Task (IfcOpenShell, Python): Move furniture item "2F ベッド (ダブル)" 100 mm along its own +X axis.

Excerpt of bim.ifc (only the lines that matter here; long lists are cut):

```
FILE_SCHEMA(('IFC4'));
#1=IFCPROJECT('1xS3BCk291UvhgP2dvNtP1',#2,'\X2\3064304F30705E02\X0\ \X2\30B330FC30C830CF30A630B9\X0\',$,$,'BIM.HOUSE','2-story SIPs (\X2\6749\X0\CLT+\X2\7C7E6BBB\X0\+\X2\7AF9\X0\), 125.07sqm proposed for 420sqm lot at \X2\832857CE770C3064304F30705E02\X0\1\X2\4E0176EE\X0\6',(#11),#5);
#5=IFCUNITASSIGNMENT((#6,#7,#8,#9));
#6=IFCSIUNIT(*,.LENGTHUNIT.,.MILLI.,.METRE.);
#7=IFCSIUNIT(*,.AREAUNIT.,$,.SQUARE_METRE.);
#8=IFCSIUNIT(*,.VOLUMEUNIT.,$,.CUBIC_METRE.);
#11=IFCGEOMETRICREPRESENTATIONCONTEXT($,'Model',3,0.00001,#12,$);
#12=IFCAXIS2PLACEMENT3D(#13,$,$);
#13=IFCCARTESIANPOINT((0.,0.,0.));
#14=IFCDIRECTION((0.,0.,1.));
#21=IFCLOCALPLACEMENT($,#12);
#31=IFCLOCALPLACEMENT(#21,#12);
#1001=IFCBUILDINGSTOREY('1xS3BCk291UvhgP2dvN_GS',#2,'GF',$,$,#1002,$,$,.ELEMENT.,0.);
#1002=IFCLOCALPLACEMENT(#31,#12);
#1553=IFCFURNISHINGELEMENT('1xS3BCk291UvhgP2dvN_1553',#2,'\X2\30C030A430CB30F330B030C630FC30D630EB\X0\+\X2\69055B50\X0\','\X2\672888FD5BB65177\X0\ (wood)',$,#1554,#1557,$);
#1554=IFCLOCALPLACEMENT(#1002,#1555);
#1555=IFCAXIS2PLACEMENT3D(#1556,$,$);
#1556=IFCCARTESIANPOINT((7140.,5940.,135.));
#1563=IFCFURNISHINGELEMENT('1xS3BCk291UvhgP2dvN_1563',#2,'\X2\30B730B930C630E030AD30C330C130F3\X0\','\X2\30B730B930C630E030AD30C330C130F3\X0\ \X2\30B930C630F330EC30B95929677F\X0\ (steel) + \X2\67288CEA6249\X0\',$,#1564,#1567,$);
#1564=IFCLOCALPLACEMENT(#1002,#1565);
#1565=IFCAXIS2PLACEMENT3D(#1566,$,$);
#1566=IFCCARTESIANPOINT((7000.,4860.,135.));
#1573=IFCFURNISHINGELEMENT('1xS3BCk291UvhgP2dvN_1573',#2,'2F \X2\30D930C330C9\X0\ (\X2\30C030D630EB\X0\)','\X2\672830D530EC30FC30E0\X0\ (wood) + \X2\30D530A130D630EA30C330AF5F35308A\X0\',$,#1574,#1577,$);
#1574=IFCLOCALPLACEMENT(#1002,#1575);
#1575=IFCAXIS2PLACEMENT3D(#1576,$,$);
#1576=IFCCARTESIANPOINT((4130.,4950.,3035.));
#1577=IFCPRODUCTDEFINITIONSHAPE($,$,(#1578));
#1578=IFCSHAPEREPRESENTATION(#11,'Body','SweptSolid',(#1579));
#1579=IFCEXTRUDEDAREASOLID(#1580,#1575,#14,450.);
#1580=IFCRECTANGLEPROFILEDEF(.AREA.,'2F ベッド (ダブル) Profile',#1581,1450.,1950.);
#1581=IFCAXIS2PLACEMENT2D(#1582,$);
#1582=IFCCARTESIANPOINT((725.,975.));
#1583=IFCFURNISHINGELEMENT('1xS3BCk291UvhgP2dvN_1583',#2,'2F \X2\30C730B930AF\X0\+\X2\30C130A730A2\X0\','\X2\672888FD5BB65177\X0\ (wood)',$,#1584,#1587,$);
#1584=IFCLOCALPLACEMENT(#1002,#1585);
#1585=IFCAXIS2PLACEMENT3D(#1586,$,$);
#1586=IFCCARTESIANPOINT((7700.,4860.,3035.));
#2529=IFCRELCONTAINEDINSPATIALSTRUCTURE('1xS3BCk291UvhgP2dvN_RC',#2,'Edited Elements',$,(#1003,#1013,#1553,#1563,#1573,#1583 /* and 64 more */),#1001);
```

```python
import ifcopenshell
import ifcopenshell.api.geometry
import ifcopenshell.util.placement
import ifcopenshell.util.unit

model = ifcopenshell.open("bim.ifc")
unit_scale = ifcopenshell.util.unit.calculate_unit_scale(model)

item = model.by_guid("1xS3BCk291UvhgP2dvN_1573")
matrix = ifcopenshell.util.placement.get_local_placement(item.ObjectPlacement)
matrix[:3, 3] += matrix[:3, 0] * 0.1 / unit_scale
ifcopenshell.api.geometry.edit_object_placement(model, product=item, matrix=matrix, is_si=False)

print(ifcopenshell.util.placement.get_local_placement(item.ObjectPlacement).round(3) + 0.0)

model.write("bim-out.ifc")
```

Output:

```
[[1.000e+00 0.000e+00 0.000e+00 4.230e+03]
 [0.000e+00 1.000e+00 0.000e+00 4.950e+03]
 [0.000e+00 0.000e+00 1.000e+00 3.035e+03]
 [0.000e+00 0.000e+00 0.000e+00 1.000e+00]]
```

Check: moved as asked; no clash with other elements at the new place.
